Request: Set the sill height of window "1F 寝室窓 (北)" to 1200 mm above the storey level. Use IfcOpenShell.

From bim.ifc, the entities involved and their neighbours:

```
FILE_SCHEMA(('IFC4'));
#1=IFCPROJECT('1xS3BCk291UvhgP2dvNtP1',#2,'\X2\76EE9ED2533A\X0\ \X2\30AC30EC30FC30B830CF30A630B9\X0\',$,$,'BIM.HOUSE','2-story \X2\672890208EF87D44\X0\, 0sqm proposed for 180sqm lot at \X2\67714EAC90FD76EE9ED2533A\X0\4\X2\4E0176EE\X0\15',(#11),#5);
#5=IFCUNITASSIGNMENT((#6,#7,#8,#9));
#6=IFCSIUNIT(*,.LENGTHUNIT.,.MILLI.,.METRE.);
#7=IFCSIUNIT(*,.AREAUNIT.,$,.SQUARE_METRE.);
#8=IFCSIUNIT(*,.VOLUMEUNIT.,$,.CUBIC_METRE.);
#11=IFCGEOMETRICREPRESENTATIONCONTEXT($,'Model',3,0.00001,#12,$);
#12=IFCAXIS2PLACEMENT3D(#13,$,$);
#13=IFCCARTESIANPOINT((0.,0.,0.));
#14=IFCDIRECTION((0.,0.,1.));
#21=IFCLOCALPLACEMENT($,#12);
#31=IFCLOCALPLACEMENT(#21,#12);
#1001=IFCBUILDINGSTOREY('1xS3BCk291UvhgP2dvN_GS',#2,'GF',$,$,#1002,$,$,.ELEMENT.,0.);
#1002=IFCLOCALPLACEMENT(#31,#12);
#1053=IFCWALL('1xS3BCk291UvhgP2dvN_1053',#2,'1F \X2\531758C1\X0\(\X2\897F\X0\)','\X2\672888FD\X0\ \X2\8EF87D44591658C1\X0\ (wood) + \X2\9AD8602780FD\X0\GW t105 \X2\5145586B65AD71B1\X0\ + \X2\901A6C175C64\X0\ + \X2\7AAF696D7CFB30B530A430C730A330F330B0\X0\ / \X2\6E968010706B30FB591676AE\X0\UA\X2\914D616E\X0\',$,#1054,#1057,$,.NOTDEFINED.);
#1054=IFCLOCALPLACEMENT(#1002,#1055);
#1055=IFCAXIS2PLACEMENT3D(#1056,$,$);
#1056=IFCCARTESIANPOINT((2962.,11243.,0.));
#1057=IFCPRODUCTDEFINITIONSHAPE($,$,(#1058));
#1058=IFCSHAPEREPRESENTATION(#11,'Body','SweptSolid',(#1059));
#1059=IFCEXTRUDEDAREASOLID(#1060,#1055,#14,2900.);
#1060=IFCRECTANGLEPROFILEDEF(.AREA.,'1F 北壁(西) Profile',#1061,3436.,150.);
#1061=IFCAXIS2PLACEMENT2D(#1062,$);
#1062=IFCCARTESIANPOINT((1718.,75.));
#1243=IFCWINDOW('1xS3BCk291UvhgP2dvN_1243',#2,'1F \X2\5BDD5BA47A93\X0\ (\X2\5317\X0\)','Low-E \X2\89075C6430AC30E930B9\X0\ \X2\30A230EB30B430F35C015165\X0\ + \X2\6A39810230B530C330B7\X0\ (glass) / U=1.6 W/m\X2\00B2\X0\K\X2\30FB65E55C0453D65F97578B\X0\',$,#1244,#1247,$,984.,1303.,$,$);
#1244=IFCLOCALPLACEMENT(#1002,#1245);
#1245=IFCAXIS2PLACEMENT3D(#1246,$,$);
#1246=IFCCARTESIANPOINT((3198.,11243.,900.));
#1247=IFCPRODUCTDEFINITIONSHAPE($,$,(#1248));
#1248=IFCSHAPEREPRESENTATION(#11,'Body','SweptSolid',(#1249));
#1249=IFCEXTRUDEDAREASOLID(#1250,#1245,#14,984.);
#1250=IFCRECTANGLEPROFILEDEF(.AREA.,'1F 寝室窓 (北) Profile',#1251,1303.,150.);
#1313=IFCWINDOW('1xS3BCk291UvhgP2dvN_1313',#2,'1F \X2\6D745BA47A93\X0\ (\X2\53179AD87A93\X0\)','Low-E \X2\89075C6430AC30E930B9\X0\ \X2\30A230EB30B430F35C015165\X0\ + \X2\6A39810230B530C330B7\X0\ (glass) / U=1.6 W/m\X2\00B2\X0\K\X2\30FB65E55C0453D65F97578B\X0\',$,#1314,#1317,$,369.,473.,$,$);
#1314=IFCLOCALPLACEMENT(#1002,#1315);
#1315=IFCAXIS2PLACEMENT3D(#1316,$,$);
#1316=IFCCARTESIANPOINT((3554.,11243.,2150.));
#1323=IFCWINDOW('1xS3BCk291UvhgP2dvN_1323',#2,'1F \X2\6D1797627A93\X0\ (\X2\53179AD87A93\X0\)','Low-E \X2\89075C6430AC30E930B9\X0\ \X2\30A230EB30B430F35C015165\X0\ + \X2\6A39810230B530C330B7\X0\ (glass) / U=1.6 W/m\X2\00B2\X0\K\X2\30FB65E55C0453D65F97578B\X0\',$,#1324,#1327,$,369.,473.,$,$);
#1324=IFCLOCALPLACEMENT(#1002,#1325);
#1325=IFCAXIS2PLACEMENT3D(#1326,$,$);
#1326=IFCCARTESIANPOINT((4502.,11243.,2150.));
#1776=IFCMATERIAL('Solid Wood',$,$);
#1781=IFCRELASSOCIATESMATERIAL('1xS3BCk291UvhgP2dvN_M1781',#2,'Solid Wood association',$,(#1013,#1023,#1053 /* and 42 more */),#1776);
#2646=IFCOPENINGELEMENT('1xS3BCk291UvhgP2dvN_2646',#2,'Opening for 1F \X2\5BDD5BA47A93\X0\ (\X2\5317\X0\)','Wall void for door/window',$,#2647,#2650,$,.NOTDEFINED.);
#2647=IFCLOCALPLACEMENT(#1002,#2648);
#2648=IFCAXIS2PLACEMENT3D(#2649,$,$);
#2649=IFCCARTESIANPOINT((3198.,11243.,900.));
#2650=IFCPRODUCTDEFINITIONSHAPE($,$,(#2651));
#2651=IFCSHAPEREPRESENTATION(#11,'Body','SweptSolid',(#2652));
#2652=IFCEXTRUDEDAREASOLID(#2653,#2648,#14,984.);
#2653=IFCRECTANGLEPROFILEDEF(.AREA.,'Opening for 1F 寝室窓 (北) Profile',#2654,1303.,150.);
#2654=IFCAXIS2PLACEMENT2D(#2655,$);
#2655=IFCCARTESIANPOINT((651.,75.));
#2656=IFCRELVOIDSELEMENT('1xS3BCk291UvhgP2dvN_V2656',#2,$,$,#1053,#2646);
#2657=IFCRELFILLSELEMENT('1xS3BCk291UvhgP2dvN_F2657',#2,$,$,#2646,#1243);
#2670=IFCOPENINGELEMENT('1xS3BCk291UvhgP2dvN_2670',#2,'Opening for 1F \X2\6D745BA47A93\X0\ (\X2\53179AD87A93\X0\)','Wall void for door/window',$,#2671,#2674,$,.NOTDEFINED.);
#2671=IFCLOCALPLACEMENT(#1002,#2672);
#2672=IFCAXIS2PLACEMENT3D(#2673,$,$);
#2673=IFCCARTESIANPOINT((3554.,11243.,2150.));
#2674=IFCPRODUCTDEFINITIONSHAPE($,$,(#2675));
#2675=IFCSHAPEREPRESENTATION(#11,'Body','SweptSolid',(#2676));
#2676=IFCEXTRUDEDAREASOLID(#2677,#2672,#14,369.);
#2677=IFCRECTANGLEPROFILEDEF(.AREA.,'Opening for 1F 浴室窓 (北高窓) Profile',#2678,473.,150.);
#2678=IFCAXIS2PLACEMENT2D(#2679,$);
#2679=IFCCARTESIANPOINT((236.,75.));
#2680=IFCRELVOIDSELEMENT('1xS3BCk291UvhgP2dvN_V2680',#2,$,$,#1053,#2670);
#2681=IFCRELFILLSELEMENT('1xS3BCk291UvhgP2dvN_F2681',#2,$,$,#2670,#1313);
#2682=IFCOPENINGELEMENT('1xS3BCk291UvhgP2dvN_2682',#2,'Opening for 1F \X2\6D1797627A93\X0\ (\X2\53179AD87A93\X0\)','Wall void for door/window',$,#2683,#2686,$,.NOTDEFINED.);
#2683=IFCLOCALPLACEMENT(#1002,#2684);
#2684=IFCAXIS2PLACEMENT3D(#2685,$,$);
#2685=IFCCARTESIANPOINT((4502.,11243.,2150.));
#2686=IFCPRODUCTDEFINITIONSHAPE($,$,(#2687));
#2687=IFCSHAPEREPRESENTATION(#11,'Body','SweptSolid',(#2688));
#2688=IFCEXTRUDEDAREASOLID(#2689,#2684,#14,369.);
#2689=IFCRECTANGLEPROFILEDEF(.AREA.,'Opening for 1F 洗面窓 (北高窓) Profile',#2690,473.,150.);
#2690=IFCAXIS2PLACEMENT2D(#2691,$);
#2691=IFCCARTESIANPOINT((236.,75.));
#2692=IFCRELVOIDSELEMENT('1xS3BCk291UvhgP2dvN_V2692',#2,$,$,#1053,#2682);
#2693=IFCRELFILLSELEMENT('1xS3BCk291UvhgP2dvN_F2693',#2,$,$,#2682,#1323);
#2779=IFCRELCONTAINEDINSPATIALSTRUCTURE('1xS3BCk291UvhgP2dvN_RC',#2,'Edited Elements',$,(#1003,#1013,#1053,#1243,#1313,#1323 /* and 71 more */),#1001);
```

```python
import numpy as np
import ifcopenshell
import ifcopenshell.api.geometry
import ifcopenshell.geom
import ifcopenshell.util.element
import ifcopenshell.util.placement
import ifcopenshell.util.shape
import ifcopenshell.util.unit

model = ifcopenshell.open("bim.ifc")
unit_scale = ifcopenshell.util.unit.calculate_unit_scale(model)

window = model.by_guid("1xS3BCk291UvhgP2dvN_1243")
opening = window.FillsVoids[0].RelatingOpeningElement
storey = ifcopenshell.util.element.get_container(window, ifc_class="IfcBuildingStorey")
level = ifcopenshell.util.placement.get_local_placement(storey.ObjectPlacement)[2, 3]

# The opening's origin need not be at the sill, so measure its lowest point.
shape = ifcopenshell.geom.create_shape(ifcopenshell.geom.settings(), opening)
bottom = ifcopenshell.util.shape.get_shape_bottom_elevation(shape, shape.geometry) / unit_scale
dz = level + 1200.0 - bottom

shift = np.array([0.0, 0.0, dz])
# The window is not placed relative to its opening, so move both.
for product in (opening, window):
    matrix = ifcopenshell.util.placement.get_local_placement(product.ObjectPlacement)
    matrix[:3, 3] += shift
    ifcopenshell.api.geometry.edit_object_placement(model, product=product, matrix=matrix, is_si=False)

print(f"moved by {dz * unit_scale:+.3f} m")

model.write("bim_edited.ifc")
```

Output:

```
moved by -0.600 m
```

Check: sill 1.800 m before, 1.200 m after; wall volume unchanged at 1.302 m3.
